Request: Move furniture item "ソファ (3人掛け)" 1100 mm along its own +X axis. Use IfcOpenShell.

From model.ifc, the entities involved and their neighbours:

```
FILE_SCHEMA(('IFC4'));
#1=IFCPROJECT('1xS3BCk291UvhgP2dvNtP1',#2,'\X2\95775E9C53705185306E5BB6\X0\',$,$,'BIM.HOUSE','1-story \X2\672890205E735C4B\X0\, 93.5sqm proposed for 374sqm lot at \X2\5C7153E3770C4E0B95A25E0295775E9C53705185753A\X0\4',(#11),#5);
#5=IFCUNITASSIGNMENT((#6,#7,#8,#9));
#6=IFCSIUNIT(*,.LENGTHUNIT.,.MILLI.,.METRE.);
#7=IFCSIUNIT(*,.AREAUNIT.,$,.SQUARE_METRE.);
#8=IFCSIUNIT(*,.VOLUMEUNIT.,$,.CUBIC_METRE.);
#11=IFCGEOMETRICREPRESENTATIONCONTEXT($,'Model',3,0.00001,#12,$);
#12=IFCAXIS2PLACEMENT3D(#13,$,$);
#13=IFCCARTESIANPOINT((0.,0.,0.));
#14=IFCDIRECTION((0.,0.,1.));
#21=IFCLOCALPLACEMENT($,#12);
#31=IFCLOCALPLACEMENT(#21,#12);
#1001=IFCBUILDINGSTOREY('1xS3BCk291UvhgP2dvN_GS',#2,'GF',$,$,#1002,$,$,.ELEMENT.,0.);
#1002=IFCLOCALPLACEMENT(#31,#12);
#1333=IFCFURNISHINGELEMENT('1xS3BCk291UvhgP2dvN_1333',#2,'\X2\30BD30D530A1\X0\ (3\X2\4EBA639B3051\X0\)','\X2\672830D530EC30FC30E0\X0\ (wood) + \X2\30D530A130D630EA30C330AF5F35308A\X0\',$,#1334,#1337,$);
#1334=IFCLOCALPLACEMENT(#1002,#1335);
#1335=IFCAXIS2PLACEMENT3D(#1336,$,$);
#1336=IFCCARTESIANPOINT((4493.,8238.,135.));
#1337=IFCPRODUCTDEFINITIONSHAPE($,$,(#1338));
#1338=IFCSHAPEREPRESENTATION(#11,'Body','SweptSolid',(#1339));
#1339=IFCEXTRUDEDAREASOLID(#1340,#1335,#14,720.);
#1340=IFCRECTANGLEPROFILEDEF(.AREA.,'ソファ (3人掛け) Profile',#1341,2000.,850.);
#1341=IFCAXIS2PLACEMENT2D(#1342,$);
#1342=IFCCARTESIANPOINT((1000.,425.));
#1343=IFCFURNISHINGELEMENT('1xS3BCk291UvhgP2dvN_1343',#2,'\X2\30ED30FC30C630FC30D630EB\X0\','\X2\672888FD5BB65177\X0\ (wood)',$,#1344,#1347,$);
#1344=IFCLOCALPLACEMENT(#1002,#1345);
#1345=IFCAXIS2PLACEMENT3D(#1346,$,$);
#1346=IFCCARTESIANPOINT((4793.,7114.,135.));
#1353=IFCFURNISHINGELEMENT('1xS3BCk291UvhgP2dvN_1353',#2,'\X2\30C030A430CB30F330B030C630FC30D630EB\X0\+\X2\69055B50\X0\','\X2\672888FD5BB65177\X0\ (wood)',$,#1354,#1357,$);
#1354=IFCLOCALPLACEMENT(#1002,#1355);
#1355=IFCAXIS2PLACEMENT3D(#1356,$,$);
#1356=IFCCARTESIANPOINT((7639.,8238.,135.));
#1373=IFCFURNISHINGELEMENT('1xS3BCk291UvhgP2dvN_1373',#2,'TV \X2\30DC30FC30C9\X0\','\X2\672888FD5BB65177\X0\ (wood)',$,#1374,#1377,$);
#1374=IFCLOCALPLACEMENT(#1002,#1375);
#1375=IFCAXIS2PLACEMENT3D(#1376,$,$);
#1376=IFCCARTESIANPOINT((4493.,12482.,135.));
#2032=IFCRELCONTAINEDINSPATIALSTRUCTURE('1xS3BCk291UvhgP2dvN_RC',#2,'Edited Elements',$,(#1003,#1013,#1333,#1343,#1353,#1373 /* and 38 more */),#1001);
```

```python
import ifcopenshell
import ifcopenshell.api.geometry
import ifcopenshell.util.placement
import ifcopenshell.util.unit

model = ifcopenshell.open("model.ifc")
unit_scale = ifcopenshell.util.unit.calculate_unit_scale(model)

item = model.by_id(1333)
matrix = ifcopenshell.util.placement.get_local_placement(item.ObjectPlacement)
matrix[:3, 3] += matrix[:3, 0] * 1.1 / unit_scale
ifcopenshell.api.geometry.edit_object_placement(model, product=item, matrix=matrix, is_si=False)

print(ifcopenshell.util.placement.get_local_placement(item.ObjectPlacement).round(3) + 0.0)

model.write("model_edited.ifc")
```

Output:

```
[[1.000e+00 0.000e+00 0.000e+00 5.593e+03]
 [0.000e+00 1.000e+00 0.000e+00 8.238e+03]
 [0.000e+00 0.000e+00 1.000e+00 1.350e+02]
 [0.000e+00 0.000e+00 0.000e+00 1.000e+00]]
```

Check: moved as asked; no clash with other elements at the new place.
